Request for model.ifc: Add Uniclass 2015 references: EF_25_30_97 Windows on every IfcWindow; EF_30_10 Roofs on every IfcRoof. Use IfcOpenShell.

First a look at what the model holds.

```python
import ifcopenshell

model = ifcopenshell.open("model.ifc")
print(model.schema)
print("classifications:", [c.Name for c in model.by_type("IfcClassification")])
for ifc_class in ("IfcDoor", "IfcRoof", "IfcStair", "IfcWall", "IfcWindow"):
    print(ifc_class, len(model.by_type(ifc_class)))
```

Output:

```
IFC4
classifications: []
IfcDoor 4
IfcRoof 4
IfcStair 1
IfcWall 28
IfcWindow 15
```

```python
import ifcopenshell
import ifcopenshell.api.classification

model = ifcopenshell.open("model.ifc")

system = ifcopenshell.api.classification.add_classification(model, classification="Uniclass 2015")

codes = {
    "IfcWindow": ("EF_25_30_97", "Windows"),
    "IfcRoof": ("EF_30_10", "Roofs"),
}
for ifc_class, (code, name) in codes.items():
    products = model.by_type(ifc_class)
    ifcopenshell.api.classification.add_reference(
        model, products=products, classification=system, identification=code, name=name
    )
    print(code, len(products))

model.write("model_updated.ifc")
```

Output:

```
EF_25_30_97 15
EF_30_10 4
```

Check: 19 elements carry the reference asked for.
